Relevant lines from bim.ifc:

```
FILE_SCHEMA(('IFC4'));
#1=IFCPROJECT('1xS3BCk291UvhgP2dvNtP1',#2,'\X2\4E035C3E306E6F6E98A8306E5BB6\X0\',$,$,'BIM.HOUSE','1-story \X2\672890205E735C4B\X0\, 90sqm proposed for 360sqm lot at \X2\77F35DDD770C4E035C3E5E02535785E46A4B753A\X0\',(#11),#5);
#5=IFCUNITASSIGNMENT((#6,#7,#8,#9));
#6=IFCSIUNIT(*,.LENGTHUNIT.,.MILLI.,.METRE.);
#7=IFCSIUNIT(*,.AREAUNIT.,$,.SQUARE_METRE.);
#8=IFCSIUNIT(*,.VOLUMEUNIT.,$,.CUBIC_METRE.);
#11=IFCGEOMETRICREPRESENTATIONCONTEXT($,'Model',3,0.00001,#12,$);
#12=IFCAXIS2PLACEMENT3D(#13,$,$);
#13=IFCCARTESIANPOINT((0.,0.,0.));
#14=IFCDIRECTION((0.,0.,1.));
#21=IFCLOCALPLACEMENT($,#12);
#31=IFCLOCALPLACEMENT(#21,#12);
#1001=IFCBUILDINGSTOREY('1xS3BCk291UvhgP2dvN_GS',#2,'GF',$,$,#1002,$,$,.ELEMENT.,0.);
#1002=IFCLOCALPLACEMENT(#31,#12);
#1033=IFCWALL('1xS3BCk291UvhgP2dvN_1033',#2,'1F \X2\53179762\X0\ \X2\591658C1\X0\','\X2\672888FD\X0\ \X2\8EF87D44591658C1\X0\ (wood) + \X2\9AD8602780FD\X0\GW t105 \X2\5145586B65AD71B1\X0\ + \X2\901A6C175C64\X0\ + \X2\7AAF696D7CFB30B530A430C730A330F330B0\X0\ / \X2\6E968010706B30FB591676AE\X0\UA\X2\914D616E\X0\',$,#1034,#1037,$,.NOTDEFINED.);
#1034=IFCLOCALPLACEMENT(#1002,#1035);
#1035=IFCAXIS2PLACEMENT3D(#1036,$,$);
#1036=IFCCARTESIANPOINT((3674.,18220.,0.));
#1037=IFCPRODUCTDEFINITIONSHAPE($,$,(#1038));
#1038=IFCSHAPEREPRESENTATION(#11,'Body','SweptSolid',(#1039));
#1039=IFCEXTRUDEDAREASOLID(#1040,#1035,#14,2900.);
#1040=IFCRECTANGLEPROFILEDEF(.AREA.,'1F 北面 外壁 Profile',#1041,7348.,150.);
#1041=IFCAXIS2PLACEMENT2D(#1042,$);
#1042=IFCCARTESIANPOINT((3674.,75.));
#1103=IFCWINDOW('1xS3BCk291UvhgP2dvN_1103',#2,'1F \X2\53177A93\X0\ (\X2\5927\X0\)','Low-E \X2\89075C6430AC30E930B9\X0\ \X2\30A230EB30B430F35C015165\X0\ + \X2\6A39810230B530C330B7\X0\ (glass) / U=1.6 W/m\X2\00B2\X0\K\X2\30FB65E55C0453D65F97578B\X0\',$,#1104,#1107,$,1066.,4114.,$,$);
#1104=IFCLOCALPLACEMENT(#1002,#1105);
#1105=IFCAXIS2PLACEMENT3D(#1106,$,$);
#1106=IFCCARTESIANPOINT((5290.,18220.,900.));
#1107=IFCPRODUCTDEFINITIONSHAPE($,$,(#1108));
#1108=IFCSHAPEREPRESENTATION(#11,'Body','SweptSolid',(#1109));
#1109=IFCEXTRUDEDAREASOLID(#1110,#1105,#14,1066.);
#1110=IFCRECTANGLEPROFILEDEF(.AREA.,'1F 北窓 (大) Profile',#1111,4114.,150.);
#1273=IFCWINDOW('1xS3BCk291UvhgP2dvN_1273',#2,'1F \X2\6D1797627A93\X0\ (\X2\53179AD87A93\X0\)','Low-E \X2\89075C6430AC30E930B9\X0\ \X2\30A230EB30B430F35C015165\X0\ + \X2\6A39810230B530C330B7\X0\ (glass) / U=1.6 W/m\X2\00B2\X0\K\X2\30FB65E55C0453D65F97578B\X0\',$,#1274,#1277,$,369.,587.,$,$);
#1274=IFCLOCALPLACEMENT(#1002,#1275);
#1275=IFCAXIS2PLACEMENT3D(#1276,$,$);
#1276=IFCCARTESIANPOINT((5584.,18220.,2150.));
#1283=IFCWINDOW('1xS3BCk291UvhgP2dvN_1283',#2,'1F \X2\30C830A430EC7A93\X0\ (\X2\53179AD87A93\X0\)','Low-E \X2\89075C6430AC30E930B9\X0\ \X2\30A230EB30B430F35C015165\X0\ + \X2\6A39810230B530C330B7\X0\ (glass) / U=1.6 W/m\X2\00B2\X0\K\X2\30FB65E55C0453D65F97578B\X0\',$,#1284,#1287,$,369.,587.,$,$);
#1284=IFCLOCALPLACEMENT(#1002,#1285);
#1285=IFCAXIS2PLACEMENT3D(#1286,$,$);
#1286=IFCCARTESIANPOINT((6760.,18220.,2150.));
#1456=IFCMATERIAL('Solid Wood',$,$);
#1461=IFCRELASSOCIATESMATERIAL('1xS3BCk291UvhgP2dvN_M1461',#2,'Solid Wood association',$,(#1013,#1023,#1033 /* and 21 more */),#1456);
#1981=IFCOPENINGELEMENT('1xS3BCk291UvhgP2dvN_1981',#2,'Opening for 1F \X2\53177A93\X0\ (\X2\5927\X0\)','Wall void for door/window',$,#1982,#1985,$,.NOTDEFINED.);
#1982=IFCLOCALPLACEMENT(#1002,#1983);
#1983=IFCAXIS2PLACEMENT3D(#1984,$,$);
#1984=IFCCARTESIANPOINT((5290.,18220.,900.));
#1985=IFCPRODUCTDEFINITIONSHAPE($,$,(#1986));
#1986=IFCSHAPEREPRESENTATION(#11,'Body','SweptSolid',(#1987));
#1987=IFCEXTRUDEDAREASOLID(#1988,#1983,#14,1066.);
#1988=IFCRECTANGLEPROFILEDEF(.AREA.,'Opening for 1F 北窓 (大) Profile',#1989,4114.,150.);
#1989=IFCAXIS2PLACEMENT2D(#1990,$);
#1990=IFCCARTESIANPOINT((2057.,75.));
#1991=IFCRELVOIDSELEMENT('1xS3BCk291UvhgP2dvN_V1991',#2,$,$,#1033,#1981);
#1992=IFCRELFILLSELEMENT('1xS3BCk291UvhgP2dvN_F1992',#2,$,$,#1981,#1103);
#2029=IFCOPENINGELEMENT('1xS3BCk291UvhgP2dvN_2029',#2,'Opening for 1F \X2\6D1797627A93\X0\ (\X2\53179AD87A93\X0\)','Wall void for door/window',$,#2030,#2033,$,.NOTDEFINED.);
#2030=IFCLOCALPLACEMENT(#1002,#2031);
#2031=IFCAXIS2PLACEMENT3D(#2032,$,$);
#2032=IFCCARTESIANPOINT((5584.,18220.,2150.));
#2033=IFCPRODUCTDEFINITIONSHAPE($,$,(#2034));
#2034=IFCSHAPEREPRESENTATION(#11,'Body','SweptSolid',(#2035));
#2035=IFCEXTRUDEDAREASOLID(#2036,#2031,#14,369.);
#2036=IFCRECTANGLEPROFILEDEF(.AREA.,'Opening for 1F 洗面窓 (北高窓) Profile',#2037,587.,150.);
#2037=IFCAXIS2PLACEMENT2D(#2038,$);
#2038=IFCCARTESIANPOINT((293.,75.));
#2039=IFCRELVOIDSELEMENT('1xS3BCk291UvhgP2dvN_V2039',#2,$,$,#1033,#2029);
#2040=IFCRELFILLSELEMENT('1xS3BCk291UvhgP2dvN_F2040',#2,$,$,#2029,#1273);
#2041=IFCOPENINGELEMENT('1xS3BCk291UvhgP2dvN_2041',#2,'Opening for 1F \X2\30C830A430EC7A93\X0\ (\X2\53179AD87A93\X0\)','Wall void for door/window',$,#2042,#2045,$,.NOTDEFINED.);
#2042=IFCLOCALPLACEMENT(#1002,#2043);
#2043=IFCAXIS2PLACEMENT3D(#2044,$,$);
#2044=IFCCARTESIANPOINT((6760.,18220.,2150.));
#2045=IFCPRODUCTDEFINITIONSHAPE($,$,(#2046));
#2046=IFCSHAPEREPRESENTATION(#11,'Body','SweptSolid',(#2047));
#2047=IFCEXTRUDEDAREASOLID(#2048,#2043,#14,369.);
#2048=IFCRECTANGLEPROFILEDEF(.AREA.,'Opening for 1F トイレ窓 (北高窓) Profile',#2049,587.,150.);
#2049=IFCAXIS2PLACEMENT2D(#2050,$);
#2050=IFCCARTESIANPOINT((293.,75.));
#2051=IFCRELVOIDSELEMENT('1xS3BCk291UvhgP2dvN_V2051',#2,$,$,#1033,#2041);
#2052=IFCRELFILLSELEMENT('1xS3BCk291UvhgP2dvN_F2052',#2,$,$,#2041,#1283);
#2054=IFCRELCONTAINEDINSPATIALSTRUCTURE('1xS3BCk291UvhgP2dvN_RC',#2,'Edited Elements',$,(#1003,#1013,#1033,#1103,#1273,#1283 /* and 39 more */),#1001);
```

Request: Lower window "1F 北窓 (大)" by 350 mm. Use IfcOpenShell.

```python
import numpy as np
import ifcopenshell
import ifcopenshell.api.geometry
import ifcopenshell.util.placement
import ifcopenshell.util.unit

model = ifcopenshell.open("bim.ifc")
unit_scale = ifcopenshell.util.unit.calculate_unit_scale(model)

window = model.by_guid("1xS3BCk291UvhgP2dvN_1103")
opening = window.FillsVoids[0].RelatingOpeningElement
dz = -0.35 / unit_scale

shift = np.array([0.0, 0.0, dz])
# The window is not placed relative to its opening, so move both.
for product in (opening, window):
    matrix = ifcopenshell.util.placement.get_local_placement(product.ObjectPlacement)
    matrix[:3, 3] += shift
    ifcopenshell.api.geometry.edit_object_placement(model, product=product, matrix=matrix, is_si=False)

print(f"moved by {dz * unit_scale:+.3f} m")

model.write("bim_updated.ifc")
```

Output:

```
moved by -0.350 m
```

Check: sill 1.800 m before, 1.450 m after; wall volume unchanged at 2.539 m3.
